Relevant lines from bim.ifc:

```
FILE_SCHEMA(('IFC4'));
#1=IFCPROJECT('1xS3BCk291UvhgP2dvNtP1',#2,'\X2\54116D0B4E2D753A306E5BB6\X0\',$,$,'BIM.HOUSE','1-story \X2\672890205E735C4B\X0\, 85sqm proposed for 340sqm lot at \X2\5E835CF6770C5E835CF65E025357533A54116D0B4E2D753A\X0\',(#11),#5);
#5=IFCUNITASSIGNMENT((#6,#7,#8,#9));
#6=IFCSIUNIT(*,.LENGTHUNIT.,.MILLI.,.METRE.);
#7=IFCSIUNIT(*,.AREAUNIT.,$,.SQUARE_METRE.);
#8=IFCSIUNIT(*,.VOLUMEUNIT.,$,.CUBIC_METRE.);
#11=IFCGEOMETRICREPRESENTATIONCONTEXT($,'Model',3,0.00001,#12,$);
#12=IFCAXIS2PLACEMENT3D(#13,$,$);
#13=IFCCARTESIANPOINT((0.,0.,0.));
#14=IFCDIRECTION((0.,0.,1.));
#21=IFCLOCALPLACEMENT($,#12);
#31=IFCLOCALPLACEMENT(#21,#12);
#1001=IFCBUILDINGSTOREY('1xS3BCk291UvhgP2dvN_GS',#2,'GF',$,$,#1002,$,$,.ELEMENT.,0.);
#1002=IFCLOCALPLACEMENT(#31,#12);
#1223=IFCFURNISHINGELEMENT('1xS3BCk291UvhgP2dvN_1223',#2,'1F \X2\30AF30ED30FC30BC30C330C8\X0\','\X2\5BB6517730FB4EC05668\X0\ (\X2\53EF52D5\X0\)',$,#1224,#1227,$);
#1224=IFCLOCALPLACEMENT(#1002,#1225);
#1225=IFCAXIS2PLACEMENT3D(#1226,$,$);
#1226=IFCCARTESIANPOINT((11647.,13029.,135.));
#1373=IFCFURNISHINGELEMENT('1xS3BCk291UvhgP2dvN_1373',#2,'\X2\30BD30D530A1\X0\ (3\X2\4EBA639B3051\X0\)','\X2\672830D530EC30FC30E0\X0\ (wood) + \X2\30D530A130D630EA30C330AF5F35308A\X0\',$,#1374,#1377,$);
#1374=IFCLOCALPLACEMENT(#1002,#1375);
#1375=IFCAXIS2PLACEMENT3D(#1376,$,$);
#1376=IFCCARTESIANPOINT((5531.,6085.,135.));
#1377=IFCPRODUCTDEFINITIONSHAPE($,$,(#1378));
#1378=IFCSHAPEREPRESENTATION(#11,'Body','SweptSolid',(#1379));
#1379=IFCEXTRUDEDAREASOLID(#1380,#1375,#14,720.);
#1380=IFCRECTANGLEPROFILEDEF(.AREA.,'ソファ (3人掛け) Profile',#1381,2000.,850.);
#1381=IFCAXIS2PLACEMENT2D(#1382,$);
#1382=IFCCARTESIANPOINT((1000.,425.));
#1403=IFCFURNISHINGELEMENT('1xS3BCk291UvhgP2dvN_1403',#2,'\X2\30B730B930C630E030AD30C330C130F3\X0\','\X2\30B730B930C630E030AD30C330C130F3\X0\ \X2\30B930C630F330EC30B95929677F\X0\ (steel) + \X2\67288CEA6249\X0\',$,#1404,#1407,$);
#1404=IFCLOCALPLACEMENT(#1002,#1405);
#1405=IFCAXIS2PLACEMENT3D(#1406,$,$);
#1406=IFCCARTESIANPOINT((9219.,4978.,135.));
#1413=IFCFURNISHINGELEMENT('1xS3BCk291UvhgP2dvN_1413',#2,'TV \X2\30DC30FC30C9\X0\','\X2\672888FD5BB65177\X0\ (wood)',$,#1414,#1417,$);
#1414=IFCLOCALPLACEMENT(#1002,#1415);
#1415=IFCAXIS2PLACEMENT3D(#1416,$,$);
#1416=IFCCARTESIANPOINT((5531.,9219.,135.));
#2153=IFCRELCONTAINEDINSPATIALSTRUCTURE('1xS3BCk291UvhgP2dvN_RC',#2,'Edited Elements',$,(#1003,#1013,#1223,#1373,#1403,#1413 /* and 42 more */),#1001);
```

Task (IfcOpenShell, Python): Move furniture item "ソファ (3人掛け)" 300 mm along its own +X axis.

```python
import ifcopenshell
import ifcopenshell.api.geometry
import ifcopenshell.util.placement

model = ifcopenshell.open("bim.ifc")

item = model.by_id(1373)
matrix = ifcopenshell.util.placement.get_local_placement(item.ObjectPlacement)
matrix[:3, 3] += matrix[:3, 0] * 300.0
ifcopenshell.api.geometry.edit_object_placement(model, product=item, matrix=matrix, is_si=False)

print(ifcopenshell.util.placement.get_local_placement(item.ObjectPlacement).round(3) + 0.0)

model.write("bim_rev.ifc")
```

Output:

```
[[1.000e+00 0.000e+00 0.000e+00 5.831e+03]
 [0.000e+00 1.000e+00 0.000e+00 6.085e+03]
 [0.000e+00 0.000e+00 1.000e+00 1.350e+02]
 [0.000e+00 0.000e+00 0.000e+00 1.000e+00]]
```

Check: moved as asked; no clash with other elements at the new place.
